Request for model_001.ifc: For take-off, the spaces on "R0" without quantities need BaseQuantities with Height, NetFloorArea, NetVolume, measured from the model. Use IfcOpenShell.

First a look at what the model holds.

```python
import ifcopenshell
import ifcopenshell.util.element
import ifcopenshell.util.unit

model = ifcopenshell.open("model_001.ifc")
print(model.schema)
for unit_type in ("LENGTHUNIT", "AREAUNIT", "VOLUMEUNIT"):
    print(unit_type, ifcopenshell.util.unit.calculate_unit_scale(model, unit_type))
storey = next(s for s in model.by_type("IfcBuildingStorey") if s.Name == "R0")
spaces = [e for e in ifcopenshell.util.element.get_decomposition(storey) if e.is_a("IfcSpace")]
for e in sorted(spaces, key=lambda e: e.id()):
    print(e.id(), e.is_a(), e.Name, list(ifcopenshell.util.element.get_psets(e, qtos_only=True)), sep=" | ")
```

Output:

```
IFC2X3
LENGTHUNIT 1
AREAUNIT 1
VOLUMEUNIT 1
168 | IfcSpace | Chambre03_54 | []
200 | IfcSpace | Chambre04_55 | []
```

```python
import ifcopenshell
import ifcopenshell.api.pset
import ifcopenshell.geom
import ifcopenshell.util.element
import ifcopenshell.util.shape
import ifcopenshell.util.unit

model = ifcopenshell.open("model_001.ifc")
unit_scale = ifcopenshell.util.unit.calculate_unit_scale(model)
area_scale = ifcopenshell.util.unit.calculate_unit_scale(model, "AREAUNIT")
volume_scale = ifcopenshell.util.unit.calculate_unit_scale(model, "VOLUMEUNIT")
settings = ifcopenshell.geom.settings()

storey = next(s for s in model.by_type("IfcBuildingStorey") if s.Name == "R0")
spaces = [e for e in ifcopenshell.util.element.get_decomposition(storey) if e.is_a("IfcSpace")]

for e in sorted(spaces, key=lambda e: e.id()):
    if ifcopenshell.util.element.get_psets(e, qtos_only=True, should_inherit=False):
        continue
    # Geometry comes back in metres, in the element's own axes.
    shape = ifcopenshell.geom.create_shape(settings, e)
    values = {
        "Height": ifcopenshell.util.shape.get_z(shape.geometry) / unit_scale,
        "NetFloorArea": ifcopenshell.util.shape.get_footprint_area(shape.geometry) / area_scale,
        "NetVolume": ifcopenshell.util.shape.get_volume(shape.geometry) / volume_scale,
    }
    qto = ifcopenshell.api.pset.add_qto(model, product=e, name="BaseQuantities")
    ifcopenshell.api.pset.edit_qto(model, qto=qto, properties=values)
    print(e.id(), {k: round(v, 3) for k, v in values.items()})

model.write("model_001-out.ifc")
```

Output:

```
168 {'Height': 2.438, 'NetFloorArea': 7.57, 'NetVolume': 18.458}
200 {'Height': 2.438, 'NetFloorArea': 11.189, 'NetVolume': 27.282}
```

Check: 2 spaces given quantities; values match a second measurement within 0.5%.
